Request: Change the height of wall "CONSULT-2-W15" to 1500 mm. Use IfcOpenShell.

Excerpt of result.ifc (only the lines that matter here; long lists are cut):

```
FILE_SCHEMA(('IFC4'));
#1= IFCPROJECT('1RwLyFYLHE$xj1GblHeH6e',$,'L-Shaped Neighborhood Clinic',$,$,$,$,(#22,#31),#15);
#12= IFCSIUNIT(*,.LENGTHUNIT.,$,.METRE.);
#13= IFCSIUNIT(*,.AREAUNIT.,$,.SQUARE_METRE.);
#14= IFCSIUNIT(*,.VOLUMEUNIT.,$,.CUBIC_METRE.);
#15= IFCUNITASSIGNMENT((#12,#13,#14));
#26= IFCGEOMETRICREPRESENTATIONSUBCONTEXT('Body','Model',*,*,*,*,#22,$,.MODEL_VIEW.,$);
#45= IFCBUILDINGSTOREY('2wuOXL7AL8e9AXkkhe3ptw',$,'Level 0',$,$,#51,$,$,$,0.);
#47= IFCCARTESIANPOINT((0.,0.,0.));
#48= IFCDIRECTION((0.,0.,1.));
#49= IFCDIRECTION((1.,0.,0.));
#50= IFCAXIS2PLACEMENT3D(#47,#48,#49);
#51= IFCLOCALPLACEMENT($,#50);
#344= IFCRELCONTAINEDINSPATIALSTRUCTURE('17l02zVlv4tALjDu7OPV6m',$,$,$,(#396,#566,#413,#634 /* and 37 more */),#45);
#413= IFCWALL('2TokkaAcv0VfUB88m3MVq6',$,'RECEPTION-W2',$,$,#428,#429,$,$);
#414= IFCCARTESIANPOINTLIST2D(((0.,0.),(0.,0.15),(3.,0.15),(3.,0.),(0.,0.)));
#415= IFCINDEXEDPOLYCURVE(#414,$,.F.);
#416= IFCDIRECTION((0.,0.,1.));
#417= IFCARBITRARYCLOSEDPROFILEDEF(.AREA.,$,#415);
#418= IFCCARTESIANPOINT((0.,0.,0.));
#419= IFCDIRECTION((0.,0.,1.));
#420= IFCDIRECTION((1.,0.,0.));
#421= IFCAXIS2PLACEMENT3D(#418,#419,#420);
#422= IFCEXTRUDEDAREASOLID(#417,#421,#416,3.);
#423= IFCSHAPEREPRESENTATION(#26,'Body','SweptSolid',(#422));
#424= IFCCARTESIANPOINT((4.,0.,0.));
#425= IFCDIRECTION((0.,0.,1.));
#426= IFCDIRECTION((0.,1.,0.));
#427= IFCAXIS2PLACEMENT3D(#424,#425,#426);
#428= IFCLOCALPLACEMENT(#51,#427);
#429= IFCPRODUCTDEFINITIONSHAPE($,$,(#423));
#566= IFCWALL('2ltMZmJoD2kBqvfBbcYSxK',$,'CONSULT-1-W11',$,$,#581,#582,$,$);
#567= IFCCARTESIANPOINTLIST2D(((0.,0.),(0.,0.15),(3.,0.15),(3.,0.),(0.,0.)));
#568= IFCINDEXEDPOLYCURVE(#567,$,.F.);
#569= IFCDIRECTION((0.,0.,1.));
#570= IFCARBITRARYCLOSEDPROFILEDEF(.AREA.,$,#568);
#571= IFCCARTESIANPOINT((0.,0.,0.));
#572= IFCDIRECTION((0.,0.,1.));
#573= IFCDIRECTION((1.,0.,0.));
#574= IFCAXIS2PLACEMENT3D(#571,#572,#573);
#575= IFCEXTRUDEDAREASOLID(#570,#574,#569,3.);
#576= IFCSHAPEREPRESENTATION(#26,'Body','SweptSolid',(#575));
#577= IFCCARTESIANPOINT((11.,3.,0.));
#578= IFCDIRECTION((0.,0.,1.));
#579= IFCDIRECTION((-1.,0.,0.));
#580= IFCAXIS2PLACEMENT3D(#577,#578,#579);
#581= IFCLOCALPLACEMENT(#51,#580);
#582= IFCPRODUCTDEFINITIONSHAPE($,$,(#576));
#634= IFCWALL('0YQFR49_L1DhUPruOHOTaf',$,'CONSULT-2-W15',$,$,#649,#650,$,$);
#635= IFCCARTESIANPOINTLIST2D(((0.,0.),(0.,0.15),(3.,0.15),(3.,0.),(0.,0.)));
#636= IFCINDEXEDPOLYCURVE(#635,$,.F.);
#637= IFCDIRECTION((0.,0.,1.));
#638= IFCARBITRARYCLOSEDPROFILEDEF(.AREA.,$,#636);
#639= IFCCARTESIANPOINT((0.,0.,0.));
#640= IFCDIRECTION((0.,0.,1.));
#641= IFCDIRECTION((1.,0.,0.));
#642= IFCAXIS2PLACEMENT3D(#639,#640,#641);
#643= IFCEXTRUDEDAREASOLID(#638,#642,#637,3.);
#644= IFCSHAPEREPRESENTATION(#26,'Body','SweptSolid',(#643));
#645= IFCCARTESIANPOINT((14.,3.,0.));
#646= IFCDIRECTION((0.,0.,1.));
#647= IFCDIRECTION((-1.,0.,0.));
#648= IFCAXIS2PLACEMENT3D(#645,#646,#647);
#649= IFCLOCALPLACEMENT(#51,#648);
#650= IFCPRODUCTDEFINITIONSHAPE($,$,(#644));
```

```python
import ifcopenshell
import ifcopenshell.geom
import ifcopenshell.util.representation
import ifcopenshell.util.shape

model = ifcopenshell.open("result.ifc")
settings = ifcopenshell.geom.settings()


def volume(element):
    """Net volume in cubic metres, openings subtracted."""
    shape = ifcopenshell.geom.create_shape(settings, element)
    return ifcopenshell.util.shape.get_volume(shape.geometry)


wall = model.by_guid("0YQFR49_L1DhUPruOHOTaf")
before = volume(wall)

body = ifcopenshell.util.representation.get_representation(wall, "Model", "Body")
solid = body.Items[0]
old_height = solid.Depth
solid.Depth = 1.5
after = volume(wall)

print(f"height {old_height:g} -> {solid.Depth:g}, volume {before:.3f} -> {after:.3f} m3")

model.write("result-out.ifc")
```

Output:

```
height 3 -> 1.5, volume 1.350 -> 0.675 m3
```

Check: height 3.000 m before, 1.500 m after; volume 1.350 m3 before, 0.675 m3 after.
